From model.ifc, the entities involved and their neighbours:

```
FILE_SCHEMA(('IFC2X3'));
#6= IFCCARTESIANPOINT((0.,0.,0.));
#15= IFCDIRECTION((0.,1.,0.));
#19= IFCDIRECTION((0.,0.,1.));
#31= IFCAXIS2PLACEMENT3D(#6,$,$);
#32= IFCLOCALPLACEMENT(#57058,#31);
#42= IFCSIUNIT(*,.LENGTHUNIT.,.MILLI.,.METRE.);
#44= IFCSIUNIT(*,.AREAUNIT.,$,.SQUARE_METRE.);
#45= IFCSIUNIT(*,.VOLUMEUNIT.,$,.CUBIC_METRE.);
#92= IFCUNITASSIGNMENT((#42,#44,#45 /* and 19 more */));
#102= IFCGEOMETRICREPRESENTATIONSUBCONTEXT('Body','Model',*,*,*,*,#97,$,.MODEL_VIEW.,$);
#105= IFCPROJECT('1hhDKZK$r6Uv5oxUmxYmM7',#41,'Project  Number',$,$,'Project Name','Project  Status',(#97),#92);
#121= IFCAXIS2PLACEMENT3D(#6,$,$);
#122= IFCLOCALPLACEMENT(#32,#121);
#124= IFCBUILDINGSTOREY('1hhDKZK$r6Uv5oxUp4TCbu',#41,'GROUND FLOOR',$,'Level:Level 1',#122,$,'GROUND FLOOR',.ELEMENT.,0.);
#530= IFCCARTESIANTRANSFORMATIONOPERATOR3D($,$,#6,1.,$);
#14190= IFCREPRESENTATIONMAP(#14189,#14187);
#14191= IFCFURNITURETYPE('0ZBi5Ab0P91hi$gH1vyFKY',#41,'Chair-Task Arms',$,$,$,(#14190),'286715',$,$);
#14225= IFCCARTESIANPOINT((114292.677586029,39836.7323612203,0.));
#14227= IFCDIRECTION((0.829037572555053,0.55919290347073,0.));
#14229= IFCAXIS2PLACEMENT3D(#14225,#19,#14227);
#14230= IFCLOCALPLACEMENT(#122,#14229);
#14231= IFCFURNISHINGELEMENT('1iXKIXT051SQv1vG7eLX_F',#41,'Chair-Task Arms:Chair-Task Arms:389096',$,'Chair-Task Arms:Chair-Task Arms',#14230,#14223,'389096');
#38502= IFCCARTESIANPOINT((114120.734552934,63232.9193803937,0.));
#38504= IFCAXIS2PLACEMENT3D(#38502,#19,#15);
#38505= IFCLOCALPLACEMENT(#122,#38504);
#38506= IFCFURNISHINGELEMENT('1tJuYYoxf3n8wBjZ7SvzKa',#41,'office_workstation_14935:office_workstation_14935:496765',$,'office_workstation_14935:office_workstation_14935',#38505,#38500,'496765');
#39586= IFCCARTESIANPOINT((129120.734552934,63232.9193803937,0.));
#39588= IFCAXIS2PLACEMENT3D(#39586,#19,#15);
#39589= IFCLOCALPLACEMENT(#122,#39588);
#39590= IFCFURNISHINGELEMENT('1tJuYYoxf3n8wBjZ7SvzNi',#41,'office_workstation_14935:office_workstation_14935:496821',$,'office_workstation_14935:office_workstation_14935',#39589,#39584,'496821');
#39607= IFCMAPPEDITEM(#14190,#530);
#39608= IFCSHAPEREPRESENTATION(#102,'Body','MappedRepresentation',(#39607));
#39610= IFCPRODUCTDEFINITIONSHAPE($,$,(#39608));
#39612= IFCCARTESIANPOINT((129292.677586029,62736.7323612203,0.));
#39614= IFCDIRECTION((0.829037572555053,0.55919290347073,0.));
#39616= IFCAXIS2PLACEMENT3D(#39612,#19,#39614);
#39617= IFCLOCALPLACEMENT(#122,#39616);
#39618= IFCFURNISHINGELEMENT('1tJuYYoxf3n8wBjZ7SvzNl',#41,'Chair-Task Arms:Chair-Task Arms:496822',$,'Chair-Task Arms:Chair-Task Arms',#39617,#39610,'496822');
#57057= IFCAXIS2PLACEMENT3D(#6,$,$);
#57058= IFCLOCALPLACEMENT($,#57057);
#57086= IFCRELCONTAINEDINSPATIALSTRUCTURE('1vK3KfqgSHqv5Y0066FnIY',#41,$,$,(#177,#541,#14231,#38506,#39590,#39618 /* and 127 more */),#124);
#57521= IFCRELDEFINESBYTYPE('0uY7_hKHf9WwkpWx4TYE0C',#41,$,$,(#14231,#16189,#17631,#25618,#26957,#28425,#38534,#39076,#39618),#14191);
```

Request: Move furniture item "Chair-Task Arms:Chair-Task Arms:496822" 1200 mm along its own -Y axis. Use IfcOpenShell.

```python
import ifcopenshell
import ifcopenshell.api.geometry
import ifcopenshell.util.placement
import ifcopenshell.util.unit

model = ifcopenshell.open("model.ifc")
unit_scale = ifcopenshell.util.unit.calculate_unit_scale(model)

item = model.by_guid("1tJuYYoxf3n8wBjZ7SvzNl")
matrix = ifcopenshell.util.placement.get_local_placement(item.ObjectPlacement)
matrix[:3, 3] -= matrix[:3, 1] * 1.2 / unit_scale
ifcopenshell.api.geometry.edit_object_placement(model, product=item, matrix=matrix, is_si=False)

print(ifcopenshell.util.placement.get_local_placement(item.ObjectPlacement).round(3) + 0.0)

model.write("model_v2.ifc")
```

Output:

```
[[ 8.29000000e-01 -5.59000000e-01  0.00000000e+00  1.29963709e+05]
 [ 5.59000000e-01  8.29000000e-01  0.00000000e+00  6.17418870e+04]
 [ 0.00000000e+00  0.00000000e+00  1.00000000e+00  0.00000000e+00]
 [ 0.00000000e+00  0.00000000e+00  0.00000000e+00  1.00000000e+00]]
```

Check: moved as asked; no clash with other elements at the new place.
